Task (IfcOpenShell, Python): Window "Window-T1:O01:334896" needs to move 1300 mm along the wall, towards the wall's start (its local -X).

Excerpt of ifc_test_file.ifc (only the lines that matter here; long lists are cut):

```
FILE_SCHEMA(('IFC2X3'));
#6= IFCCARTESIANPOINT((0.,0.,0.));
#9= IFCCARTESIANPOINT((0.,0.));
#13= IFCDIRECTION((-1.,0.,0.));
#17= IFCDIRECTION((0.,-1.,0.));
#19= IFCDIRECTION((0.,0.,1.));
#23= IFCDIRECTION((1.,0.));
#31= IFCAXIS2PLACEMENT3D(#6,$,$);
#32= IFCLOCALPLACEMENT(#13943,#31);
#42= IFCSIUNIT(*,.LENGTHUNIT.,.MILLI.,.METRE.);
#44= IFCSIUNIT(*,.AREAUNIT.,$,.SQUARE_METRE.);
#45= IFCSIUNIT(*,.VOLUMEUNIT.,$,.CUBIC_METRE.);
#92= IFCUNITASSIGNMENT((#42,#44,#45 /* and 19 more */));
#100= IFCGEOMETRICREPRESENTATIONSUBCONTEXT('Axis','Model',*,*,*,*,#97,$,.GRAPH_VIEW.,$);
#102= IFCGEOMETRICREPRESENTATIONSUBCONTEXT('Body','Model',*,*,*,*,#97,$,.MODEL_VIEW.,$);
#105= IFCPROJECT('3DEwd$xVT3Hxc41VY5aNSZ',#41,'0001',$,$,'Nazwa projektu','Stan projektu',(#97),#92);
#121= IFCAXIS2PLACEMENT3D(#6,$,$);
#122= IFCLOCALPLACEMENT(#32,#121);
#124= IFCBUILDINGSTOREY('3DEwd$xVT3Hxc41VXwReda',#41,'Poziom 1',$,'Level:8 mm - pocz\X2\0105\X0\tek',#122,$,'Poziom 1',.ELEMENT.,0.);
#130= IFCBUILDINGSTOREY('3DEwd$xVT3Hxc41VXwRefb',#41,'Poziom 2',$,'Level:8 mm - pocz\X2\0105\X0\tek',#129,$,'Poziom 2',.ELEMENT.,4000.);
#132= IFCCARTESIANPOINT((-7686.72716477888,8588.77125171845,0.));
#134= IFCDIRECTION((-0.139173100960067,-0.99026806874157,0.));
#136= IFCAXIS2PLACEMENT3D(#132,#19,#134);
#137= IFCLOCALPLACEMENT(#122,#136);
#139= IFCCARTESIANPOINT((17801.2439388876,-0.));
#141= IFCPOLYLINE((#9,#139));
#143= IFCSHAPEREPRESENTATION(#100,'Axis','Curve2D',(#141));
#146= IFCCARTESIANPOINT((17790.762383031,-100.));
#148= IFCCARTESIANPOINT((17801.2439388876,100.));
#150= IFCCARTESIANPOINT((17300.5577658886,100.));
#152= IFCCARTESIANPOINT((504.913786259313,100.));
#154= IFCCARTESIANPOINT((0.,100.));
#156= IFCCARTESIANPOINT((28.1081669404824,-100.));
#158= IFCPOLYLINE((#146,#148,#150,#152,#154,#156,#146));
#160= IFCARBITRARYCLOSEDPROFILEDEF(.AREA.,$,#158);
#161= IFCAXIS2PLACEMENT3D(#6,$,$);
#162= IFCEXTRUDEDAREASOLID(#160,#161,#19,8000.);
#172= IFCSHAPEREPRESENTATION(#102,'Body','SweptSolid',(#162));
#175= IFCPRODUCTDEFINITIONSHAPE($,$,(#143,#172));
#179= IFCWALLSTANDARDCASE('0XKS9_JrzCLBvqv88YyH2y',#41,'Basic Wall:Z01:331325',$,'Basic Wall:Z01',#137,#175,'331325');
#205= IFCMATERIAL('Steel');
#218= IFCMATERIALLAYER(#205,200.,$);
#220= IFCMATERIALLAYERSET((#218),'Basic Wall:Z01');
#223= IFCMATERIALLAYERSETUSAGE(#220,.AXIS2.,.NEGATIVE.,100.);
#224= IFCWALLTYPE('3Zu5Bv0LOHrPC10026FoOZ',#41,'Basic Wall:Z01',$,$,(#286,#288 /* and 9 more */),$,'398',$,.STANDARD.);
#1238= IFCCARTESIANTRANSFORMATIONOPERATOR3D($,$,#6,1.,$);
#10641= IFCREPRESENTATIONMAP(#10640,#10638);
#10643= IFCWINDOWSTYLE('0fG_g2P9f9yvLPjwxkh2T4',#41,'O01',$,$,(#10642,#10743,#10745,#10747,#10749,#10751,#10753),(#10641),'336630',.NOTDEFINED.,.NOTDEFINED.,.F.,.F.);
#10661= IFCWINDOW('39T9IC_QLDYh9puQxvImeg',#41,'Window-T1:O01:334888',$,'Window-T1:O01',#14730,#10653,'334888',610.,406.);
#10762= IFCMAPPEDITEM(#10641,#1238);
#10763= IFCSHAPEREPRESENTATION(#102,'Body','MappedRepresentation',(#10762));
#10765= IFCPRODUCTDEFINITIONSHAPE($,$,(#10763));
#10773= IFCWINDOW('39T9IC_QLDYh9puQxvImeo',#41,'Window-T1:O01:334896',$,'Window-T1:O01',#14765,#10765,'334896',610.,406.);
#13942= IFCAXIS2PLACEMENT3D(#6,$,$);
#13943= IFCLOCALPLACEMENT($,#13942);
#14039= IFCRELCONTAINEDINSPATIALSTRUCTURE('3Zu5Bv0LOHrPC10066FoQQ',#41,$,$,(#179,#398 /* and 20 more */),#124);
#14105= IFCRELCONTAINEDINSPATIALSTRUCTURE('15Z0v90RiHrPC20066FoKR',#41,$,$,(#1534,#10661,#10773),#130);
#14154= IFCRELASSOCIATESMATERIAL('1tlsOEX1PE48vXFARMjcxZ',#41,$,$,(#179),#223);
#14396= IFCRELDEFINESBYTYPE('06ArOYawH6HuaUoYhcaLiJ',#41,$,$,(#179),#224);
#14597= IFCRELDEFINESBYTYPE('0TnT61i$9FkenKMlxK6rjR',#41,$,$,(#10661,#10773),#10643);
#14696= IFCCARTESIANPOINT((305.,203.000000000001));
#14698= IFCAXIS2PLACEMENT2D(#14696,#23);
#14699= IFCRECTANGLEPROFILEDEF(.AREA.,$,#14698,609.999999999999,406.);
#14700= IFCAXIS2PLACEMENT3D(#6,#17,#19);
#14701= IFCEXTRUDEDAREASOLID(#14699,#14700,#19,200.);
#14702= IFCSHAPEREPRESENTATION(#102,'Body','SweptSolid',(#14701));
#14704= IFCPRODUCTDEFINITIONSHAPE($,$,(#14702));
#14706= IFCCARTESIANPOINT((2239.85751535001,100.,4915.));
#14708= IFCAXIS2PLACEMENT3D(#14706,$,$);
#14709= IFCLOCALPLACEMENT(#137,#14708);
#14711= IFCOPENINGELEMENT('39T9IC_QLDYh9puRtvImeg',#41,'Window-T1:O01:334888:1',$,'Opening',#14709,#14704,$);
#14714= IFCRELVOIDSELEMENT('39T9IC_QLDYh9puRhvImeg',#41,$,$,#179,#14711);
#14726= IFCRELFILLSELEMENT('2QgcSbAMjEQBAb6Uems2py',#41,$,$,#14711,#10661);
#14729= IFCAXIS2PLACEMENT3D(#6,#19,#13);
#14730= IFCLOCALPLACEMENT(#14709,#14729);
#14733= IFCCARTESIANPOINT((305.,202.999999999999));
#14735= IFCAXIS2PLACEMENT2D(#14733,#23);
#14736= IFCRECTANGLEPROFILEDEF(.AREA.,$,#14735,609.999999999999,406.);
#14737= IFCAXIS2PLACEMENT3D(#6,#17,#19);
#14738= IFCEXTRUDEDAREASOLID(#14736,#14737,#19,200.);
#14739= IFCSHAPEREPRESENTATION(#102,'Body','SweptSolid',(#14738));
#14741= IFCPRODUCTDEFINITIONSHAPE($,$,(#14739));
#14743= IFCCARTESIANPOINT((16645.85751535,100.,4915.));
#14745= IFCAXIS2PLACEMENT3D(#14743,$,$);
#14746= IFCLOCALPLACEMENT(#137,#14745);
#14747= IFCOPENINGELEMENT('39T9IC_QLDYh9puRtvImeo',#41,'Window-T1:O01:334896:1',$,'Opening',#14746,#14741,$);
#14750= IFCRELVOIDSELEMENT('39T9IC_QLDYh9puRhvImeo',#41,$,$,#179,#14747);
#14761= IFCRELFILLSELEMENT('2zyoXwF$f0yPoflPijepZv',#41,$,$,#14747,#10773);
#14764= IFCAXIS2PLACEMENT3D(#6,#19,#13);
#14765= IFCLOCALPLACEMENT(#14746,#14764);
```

```python
import ifcopenshell
import ifcopenshell.api.geometry
import ifcopenshell.util.placement

model = ifcopenshell.open("ifc_test_file.ifc")

window = model.by_guid("39T9IC_QLDYh9puQxvImeo")
opening = window.FillsVoids[0].RelatingOpeningElement
wall = opening.VoidsElements[0].RelatingBuildingElement

wall_matrix = ifcopenshell.util.placement.get_local_placement(wall.ObjectPlacement)
shift = wall_matrix[:3, 0] * -1300.0
before = ifcopenshell.util.placement.get_local_placement(window.ObjectPlacement)[:3, 3].copy()

# The window is placed relative to its opening, so it follows when the opening moves.
matrix = ifcopenshell.util.placement.get_local_placement(opening.ObjectPlacement)
matrix[:3, 3] += shift
ifcopenshell.api.geometry.edit_object_placement(
    model, product=opening, matrix=matrix, is_si=False, should_transform_children=True
)

after = ifcopenshell.util.placement.get_local_placement(window.ObjectPlacement)[:3, 3]
print("window moved by", (after - before).round(3) + 0.0)

model.write("ifc_test_file_rev.ifc")
```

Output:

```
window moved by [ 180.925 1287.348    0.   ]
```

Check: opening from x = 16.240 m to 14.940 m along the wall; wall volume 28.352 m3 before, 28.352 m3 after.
